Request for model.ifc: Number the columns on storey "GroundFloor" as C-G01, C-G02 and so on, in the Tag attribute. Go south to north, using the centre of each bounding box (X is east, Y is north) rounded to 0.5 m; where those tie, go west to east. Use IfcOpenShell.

First a look at what the model holds.

```python
import ifcopenshell
import ifcopenshell.util.element
import ifcopenshell.util.placement

model = ifcopenshell.open("model.ifc")
print(model.schema)
storey = next(s for s in model.by_type("IfcBuildingStorey") if s.Name == "GroundFloor")
columns = [e for e in ifcopenshell.util.element.get_decomposition(storey) if e.is_a("IfcColumn")]
for e in sorted(columns, key=lambda e: e.id()):
    origin = ifcopenshell.util.placement.get_local_placement(e.ObjectPlacement)[:3, 3]
    print(e.id(), e.Tag, e.Name, origin.round(2) + 0.0, sep=" | ")
```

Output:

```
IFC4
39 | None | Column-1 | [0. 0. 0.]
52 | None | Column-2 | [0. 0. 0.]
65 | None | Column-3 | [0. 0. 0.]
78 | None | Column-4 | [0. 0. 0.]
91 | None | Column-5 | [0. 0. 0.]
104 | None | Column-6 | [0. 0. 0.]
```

```python
import ifcopenshell
import ifcopenshell.geom
import ifcopenshell.util.element
import ifcopenshell.util.shape

model = ifcopenshell.open("model.ifc")
settings = ifcopenshell.geom.settings()
settings.set("use-world-coords", True)


def centre(element):
    shape = ifcopenshell.geom.create_shape(settings, element)
    return ifcopenshell.util.shape.get_bbox_centroid(shape.geometry)


storey = next(s for s in model.by_type("IfcBuildingStorey") if s.Name == "GroundFloor")
columns = [e for e in ifcopenshell.util.element.get_decomposition(storey) if e.is_a("IfcColumn")]

# Insertion points can sit at a corner or the storey origin, so sort by the geometry (in metres).
centres = {e: centre(e) for e in columns}
columns.sort(key=lambda e: (round(centres[e][1] / 0.5), centres[e][0]))

for i, e in enumerate(columns, start=1):
    number = f"C-G{i:02d}"
    e.Tag = number
    print(e.id(), number)

model.write("model_updated.ifc")
```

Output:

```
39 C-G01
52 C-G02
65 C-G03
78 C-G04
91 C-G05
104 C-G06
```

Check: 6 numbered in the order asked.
